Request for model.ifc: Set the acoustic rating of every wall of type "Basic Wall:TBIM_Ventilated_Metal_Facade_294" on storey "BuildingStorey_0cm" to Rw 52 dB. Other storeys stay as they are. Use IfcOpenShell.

First a look at what the model holds.

```python
import ifcopenshell
import ifcopenshell.util.element

model = ifcopenshell.open("model.ifc")
print(model.schema)
storey = next(s for s in model.by_type("IfcBuildingStorey") if s.Name == "BuildingStorey_0cm")
walls = [e for e in ifcopenshell.util.element.get_decomposition(storey) if e.is_a("IfcWall")]
seen = {}
for e in walls:
    element_type = ifcopenshell.util.element.get_type(e)
    key = (element_type.Name if element_type != e and element_type else None, ifcopenshell.util.element.get_pset(e, "Pset_WallCommon", "AcousticRating"))
    seen[key] = seen.get(key, 0) + 1
for (name, value), count in sorted(seen.items(), key=str):
    print(count, "x", name, "|", value)
```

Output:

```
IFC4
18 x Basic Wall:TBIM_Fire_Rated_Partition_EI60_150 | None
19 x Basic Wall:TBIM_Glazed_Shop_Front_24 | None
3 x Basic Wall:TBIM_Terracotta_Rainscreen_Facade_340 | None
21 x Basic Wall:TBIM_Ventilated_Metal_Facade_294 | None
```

```python
import ifcopenshell
import ifcopenshell.api.pset
import ifcopenshell.util.element

model = ifcopenshell.open("model.ifc")

storey = next(s for s in model.by_type("IfcBuildingStorey") if s.Name == "BuildingStorey_0cm")
walls = [e for e in ifcopenshell.util.element.get_decomposition(storey) if e.is_a("IfcWall")]

count = 0
for e in walls:
    element_type = ifcopenshell.util.element.get_type(e)
    if element_type in (None, e) or element_type.Name != "Basic Wall:TBIM_Ventilated_Metal_Facade_294":
        continue
    # add_pset returns the element's existing set when there is one.
    pset = ifcopenshell.api.pset.add_pset(model, product=e, name="Pset_WallCommon")
    ifcopenshell.api.pset.edit_pset(model, pset=pset, properties={"AcousticRating": "Rw 52 dB"})
    count += 1

print(count, "walls updated")

model.write("model_v2.ifc")
```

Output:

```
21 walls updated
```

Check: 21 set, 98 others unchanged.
